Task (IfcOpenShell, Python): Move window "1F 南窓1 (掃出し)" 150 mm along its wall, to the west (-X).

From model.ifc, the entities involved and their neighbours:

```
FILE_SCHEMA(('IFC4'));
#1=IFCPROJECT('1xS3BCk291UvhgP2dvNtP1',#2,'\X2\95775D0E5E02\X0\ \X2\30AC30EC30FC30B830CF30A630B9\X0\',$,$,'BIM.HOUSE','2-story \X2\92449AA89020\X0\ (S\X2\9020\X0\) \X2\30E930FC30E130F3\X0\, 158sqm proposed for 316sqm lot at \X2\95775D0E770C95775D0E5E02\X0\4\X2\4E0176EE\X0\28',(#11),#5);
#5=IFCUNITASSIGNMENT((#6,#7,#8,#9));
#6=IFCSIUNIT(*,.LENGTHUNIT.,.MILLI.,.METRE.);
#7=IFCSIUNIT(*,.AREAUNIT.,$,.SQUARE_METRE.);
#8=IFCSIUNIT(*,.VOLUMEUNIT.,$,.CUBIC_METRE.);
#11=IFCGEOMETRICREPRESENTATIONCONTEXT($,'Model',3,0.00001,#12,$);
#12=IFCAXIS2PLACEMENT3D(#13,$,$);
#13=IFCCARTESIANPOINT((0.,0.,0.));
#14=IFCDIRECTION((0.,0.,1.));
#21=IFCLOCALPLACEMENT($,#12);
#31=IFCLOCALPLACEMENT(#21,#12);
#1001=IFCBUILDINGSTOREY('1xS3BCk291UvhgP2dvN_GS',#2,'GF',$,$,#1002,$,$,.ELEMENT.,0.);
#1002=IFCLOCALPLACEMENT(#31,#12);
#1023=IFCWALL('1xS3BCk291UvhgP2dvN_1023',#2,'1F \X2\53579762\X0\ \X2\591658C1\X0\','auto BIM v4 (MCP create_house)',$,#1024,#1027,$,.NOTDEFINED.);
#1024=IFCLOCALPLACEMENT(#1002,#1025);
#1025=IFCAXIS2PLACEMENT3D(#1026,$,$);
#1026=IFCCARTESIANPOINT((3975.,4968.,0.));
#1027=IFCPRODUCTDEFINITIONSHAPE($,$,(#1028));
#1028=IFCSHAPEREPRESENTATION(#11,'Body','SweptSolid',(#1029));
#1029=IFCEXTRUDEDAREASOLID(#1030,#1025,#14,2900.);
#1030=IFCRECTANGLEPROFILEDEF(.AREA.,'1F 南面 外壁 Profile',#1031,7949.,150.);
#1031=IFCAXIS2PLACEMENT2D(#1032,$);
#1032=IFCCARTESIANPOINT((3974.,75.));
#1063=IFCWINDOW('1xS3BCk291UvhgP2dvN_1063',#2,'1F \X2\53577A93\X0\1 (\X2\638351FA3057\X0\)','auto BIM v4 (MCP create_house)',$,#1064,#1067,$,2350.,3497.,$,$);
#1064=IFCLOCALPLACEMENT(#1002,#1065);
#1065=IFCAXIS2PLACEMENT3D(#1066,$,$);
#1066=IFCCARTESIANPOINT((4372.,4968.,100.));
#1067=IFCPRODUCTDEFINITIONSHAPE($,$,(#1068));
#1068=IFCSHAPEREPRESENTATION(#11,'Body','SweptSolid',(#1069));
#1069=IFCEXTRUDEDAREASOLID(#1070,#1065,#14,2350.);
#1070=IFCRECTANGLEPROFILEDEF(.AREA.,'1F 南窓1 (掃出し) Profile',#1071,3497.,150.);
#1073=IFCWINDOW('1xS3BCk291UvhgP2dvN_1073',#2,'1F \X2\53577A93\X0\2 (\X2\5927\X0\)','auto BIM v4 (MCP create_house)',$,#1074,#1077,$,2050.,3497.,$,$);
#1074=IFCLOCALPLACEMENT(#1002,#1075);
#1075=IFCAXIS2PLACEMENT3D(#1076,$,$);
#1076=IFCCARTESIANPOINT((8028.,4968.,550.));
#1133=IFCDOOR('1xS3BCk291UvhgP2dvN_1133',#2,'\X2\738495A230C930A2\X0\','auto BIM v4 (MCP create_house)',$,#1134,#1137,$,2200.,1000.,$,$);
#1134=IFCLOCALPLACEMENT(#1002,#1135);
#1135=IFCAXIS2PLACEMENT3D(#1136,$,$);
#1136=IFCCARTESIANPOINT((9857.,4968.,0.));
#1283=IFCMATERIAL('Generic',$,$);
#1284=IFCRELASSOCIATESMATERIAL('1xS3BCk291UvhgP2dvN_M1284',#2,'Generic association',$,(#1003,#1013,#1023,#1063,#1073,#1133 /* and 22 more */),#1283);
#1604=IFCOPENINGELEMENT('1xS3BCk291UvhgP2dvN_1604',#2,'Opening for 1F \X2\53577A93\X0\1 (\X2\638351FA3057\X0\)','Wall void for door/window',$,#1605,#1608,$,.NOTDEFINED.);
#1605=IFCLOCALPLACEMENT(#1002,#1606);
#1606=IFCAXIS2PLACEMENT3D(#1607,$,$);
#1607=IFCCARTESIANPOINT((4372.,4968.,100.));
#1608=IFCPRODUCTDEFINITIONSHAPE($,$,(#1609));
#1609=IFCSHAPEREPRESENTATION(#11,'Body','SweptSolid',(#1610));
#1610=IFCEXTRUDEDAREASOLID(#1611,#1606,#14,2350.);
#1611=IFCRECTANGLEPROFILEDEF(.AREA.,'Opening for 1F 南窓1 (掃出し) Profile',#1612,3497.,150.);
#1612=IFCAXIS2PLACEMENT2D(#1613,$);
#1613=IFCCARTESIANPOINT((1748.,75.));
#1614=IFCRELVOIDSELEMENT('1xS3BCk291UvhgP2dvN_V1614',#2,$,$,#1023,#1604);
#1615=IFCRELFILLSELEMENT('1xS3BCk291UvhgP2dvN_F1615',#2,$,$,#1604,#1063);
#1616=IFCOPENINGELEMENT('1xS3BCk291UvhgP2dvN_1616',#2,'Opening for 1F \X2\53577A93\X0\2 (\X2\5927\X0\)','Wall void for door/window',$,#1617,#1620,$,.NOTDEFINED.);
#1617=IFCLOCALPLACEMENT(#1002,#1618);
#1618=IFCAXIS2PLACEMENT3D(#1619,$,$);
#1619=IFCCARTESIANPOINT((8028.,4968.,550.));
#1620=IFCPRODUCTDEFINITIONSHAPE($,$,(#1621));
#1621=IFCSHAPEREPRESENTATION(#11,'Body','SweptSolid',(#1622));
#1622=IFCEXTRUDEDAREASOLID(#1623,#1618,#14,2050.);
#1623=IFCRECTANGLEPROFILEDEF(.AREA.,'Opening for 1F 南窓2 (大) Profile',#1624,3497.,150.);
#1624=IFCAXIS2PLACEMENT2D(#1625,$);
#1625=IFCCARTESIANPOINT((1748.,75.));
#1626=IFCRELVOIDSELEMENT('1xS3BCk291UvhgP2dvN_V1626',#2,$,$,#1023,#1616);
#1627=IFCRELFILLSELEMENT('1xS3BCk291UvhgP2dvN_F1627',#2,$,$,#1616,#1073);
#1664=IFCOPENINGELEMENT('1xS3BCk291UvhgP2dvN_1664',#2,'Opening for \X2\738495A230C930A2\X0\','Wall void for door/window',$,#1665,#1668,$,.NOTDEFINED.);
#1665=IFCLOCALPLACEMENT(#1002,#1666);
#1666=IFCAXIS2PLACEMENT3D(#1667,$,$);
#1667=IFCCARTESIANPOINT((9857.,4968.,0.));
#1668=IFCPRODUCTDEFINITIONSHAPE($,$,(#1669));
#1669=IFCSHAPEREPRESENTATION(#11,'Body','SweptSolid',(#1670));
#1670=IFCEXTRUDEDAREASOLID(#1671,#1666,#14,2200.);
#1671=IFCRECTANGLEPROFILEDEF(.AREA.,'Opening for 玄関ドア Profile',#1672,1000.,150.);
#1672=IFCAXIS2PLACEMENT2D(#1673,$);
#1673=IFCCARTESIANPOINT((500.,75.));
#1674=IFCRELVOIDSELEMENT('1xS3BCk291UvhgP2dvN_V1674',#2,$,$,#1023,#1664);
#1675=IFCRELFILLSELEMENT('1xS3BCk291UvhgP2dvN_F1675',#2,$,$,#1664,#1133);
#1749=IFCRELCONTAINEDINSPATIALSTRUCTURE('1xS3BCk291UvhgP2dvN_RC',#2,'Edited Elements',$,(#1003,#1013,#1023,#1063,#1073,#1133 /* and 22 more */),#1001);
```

```python
import ifcopenshell
import ifcopenshell.api.geometry
import ifcopenshell.util.placement
import ifcopenshell.util.unit

model = ifcopenshell.open("model.ifc")
unit_scale = ifcopenshell.util.unit.calculate_unit_scale(model)

window = model.by_guid("1xS3BCk291UvhgP2dvN_1063")
opening = window.FillsVoids[0].RelatingOpeningElement
wall = opening.VoidsElements[0].RelatingBuildingElement

wall_matrix = ifcopenshell.util.placement.get_local_placement(wall.ObjectPlacement)
shift = wall_matrix[:3, 0] * -0.15 / unit_scale
before = ifcopenshell.util.placement.get_local_placement(window.ObjectPlacement)[:3, 3].copy()

# The window is not placed relative to its opening, so move both.
for product in (opening, window):
    matrix = ifcopenshell.util.placement.get_local_placement(product.ObjectPlacement)
    matrix[:3, 3] += shift
    ifcopenshell.api.geometry.edit_object_placement(model, product=product, matrix=matrix, is_si=False)

after = ifcopenshell.util.placement.get_local_placement(window.ObjectPlacement)[:3, 3]
print("window moved by", (after - before).round(3) + 0.0)

model.write("model_rev.ifc")
```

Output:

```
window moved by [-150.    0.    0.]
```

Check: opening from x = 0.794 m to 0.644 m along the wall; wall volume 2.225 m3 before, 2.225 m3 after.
